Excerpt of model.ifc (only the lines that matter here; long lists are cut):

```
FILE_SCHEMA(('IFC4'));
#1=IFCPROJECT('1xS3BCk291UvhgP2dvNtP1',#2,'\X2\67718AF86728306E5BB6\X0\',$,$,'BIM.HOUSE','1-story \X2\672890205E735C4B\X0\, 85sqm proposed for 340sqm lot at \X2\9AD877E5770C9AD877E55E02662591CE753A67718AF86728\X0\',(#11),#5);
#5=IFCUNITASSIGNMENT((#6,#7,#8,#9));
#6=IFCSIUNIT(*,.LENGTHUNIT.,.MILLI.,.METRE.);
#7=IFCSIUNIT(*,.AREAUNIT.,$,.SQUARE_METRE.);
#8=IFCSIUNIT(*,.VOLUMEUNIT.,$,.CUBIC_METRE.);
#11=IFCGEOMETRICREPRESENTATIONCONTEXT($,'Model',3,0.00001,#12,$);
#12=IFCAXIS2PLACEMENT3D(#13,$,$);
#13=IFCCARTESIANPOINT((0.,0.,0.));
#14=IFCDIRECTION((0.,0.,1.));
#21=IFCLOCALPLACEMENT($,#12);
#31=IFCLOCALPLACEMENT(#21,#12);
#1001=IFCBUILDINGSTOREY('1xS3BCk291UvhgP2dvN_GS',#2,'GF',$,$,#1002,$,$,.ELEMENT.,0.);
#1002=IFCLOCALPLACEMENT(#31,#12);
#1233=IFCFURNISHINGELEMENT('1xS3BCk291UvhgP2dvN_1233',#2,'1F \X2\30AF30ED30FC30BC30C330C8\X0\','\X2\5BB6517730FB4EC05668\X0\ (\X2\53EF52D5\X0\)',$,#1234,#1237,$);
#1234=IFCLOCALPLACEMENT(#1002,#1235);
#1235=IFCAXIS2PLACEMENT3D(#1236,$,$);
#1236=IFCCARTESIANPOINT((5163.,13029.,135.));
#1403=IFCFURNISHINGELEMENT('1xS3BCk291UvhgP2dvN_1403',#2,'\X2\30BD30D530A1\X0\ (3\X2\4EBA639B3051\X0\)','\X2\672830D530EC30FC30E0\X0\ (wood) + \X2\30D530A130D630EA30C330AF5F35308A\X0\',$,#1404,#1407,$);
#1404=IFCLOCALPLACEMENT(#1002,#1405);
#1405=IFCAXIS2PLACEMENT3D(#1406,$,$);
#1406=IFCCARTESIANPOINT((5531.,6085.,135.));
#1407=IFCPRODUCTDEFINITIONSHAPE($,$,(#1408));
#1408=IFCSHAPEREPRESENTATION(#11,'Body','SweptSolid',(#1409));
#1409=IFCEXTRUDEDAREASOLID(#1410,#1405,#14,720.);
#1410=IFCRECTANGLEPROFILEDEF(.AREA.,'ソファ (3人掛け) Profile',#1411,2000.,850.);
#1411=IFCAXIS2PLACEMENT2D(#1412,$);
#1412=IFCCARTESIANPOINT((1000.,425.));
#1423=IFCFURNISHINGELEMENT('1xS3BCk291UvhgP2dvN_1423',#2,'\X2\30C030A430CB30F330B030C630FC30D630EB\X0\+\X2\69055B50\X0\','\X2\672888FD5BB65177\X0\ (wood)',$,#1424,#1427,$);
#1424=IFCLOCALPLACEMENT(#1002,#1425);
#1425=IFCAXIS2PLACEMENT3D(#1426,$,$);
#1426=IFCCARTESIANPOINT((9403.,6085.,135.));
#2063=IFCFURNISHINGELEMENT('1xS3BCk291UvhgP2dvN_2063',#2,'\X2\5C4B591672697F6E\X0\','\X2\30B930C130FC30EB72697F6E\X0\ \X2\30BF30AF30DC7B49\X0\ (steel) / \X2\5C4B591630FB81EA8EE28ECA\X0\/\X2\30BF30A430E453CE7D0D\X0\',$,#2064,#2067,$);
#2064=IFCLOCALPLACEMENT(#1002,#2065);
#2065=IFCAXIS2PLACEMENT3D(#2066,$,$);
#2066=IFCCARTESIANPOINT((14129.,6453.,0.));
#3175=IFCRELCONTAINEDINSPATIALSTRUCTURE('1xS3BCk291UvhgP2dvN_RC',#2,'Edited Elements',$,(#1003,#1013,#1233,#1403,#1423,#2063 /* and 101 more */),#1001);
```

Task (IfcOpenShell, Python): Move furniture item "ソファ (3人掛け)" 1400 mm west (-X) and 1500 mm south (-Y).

```python
import ifcopenshell
import ifcopenshell.api.geometry
import ifcopenshell.util.placement
import ifcopenshell.util.unit

model = ifcopenshell.open("model.ifc")
unit_scale = ifcopenshell.util.unit.calculate_unit_scale(model)

item = model.by_guid("1xS3BCk291UvhgP2dvN_1403")
matrix = ifcopenshell.util.placement.get_local_placement(item.ObjectPlacement)
matrix[0, 3] -= 1.4 / unit_scale
matrix[1, 3] -= 1.5 / unit_scale
ifcopenshell.api.geometry.edit_object_placement(model, product=item, matrix=matrix, is_si=False)

print(ifcopenshell.util.placement.get_local_placement(item.ObjectPlacement).round(3) + 0.0)

model.write("model_rev.ifc")
```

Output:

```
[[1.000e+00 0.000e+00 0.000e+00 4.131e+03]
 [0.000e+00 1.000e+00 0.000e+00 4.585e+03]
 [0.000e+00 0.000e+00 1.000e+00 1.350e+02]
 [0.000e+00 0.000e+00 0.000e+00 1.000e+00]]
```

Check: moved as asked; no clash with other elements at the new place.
